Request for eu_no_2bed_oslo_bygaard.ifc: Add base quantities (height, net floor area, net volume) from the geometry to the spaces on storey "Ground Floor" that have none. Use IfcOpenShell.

First a look at what the model holds.

```python
import ifcopenshell
import ifcopenshell.util.element
import ifcopenshell.util.unit

model = ifcopenshell.open("eu_no_2bed_oslo_bygaard.ifc")
print(model.schema)
for unit_type in ("LENGTHUNIT", "AREAUNIT", "VOLUMEUNIT"):
    print(unit_type, ifcopenshell.util.unit.calculate_unit_scale(model, unit_type))
storey = next(s for s in model.by_type("IfcBuildingStorey") if s.Name == "Ground Floor")
spaces = [e for e in ifcopenshell.util.element.get_decomposition(storey) if e.is_a("IfcSpace")]
for e in sorted(spaces, key=lambda e: e.id()):
    print(e.id(), e.is_a(), e.Name, list(ifcopenshell.util.element.get_psets(e, qtos_only=True)), sep=" | ")
```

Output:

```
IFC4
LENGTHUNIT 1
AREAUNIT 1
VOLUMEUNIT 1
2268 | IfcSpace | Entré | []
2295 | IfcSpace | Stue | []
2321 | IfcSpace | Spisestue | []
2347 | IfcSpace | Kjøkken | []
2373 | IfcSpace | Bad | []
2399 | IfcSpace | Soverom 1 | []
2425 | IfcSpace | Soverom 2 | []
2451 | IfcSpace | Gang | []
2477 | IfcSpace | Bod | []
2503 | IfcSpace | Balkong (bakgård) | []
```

```python
import ifcopenshell
import ifcopenshell.api.pset
import ifcopenshell.geom
import ifcopenshell.util.element
import ifcopenshell.util.shape
import ifcopenshell.util.unit

model = ifcopenshell.open("eu_no_2bed_oslo_bygaard.ifc")
unit_scale = ifcopenshell.util.unit.calculate_unit_scale(model)
area_scale = ifcopenshell.util.unit.calculate_unit_scale(model, "AREAUNIT")
volume_scale = ifcopenshell.util.unit.calculate_unit_scale(model, "VOLUMEUNIT")
settings = ifcopenshell.geom.settings()

storey = next(s for s in model.by_type("IfcBuildingStorey") if s.Name == "Ground Floor")
spaces = [e for e in ifcopenshell.util.element.get_decomposition(storey) if e.is_a("IfcSpace")]

for e in sorted(spaces, key=lambda e: e.id()):
    if ifcopenshell.util.element.get_psets(e, qtos_only=True, should_inherit=False):
        continue
    # Geometry comes back in metres, in the element's own axes.
    shape = ifcopenshell.geom.create_shape(settings, e)
    values = {
        "Height": ifcopenshell.util.shape.get_z(shape.geometry) / unit_scale,
        "NetFloorArea": ifcopenshell.util.shape.get_footprint_area(shape.geometry) / area_scale,
        "NetVolume": ifcopenshell.util.shape.get_volume(shape.geometry) / volume_scale,
    }
    qto = ifcopenshell.api.pset.add_qto(model, product=e, name="Qto_SpaceBaseQuantities")
    ifcopenshell.api.pset.edit_qto(model, qto=qto, properties=values)
    print(e.id(), {k: round(v, 3) for k, v in values.items()})

model.write("eu_no_2bed_oslo_bygaard_rev.ifc")
```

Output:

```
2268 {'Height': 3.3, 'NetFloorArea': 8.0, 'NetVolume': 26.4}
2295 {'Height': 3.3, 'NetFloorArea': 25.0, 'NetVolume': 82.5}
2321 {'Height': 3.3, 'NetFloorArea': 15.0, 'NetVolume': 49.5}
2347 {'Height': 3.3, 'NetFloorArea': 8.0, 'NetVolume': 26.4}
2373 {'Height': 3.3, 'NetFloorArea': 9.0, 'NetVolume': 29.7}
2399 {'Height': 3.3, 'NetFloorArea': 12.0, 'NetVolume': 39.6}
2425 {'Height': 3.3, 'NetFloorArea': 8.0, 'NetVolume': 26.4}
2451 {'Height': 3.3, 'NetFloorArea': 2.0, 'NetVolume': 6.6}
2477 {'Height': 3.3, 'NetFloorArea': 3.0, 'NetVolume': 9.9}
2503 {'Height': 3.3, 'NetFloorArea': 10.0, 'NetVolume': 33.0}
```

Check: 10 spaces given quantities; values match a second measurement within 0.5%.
